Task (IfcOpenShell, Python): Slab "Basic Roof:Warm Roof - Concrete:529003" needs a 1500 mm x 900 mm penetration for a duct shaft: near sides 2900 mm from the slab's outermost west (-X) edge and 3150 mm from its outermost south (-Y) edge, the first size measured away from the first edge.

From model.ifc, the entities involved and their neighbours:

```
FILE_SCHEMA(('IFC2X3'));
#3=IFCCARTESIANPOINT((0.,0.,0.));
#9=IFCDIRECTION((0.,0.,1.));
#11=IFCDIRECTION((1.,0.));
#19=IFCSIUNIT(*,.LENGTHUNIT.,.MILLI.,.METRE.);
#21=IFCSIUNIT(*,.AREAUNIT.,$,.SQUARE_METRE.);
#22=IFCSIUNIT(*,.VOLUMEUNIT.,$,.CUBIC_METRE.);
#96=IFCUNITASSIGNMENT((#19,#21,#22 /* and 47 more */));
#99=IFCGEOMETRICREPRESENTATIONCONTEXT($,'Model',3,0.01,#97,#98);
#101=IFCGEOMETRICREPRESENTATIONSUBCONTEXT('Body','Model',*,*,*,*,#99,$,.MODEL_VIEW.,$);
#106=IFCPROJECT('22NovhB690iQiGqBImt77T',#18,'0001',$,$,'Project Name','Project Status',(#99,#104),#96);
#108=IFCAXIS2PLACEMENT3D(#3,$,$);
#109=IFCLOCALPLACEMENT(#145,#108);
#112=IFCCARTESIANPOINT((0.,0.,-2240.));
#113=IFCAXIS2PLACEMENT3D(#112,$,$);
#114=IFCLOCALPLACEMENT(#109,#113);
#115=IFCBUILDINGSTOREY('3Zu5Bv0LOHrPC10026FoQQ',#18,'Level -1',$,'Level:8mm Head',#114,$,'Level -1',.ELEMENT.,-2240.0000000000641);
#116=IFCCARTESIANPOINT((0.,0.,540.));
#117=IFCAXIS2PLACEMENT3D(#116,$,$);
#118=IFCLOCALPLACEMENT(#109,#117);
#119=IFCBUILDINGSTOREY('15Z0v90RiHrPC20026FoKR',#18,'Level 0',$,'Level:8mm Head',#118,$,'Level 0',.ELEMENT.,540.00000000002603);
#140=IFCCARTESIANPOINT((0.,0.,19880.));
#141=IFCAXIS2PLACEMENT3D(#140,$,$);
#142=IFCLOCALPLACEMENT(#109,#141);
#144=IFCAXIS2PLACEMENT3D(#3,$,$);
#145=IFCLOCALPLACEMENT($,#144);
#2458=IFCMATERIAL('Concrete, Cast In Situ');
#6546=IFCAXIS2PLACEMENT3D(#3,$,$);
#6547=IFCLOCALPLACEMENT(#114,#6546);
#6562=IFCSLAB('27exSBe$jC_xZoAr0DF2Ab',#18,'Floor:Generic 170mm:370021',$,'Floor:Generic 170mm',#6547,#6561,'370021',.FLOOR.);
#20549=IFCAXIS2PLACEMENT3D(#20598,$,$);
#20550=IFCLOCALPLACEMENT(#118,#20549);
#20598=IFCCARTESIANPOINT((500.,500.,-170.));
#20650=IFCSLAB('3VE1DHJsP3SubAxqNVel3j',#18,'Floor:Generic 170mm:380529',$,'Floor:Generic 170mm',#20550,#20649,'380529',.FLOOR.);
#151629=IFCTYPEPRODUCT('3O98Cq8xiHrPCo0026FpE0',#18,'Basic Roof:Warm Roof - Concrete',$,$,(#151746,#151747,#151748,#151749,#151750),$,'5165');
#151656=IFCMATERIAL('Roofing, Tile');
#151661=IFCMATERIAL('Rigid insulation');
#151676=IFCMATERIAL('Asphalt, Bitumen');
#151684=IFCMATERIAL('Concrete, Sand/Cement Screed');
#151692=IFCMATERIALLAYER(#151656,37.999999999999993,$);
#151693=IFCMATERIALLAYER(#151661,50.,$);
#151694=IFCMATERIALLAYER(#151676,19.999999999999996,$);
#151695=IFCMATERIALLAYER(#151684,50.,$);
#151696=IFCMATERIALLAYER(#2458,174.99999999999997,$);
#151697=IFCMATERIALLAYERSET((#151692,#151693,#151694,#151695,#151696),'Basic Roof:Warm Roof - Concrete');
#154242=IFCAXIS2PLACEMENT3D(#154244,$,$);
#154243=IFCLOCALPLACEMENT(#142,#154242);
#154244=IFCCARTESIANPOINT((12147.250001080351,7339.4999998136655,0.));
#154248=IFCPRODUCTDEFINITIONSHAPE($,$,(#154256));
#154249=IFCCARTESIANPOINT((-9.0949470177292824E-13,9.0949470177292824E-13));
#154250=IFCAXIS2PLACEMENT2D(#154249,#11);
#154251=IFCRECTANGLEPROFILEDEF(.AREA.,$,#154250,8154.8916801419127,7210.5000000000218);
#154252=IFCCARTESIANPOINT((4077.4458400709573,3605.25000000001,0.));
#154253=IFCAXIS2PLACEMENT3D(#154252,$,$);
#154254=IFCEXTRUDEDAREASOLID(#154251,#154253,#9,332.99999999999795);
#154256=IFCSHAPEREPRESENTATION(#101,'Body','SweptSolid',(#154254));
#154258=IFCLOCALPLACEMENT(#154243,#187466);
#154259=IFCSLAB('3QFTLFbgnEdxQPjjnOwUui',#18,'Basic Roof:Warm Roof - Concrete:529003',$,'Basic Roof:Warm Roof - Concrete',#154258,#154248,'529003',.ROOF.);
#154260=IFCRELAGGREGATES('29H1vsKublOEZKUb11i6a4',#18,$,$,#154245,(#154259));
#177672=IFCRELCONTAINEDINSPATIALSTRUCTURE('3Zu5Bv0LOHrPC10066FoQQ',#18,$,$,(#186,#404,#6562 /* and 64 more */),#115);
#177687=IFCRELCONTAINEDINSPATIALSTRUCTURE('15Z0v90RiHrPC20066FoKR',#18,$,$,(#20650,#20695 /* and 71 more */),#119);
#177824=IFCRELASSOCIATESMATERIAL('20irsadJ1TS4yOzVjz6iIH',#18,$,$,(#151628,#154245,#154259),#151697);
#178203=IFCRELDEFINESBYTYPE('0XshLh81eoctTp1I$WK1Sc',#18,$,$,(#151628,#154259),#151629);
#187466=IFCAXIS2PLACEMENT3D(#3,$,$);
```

```python
import numpy as np
import ifcopenshell
import ifcopenshell.api.feature
import ifcopenshell.api.geometry
import ifcopenshell.api.root
import ifcopenshell.geom
import ifcopenshell.util.placement
import ifcopenshell.util.representation
import ifcopenshell.util.shape
import ifcopenshell.util.unit

model = ifcopenshell.open("model.ifc")
unit_scale = ifcopenshell.util.unit.calculate_unit_scale(model)
settings = ifcopenshell.geom.settings()


def volume(element):
    """Net volume in cubic metres, openings subtracted."""
    shape = ifcopenshell.geom.create_shape(settings, element)
    return ifcopenshell.util.shape.get_volume(shape.geometry)


slab = model.by_id(154259)
before = volume(slab)

# Extent in the slab's own axes, in metres. The edges named are its -X and -Y sides.
slab_shape = ifcopenshell.geom.create_shape(settings, slab)
vertices = ifcopenshell.util.shape.get_vertices(slab_shape.geometry)
x_min, y_min, bottom = vertices.min(axis=0)
top = vertices[:, 2].max()

opening = ifcopenshell.api.root.create_entity(model, ifc_class="IfcOpeningElement", name="Duct shaft opening")
context = ifcopenshell.util.representation.get_context(model, "Model", "Body", "MODEL_VIEW")
width, depth = 1.5, 0.9
outline = [(0.0, 0.0), (width, 0.0), (width, depth), (0.0, depth), (0.0, 0.0)]
# Overshoot both faces by 50 mm so the cut is clean.
shape = ifcopenshell.api.geometry.add_slab_representation(
    model, context=context, depth=top - bottom + 0.1, polyline=outline
)
ifcopenshell.api.geometry.assign_representation(model, product=opening, representation=shape)

matrix = ifcopenshell.util.placement.get_local_placement(slab.ObjectPlacement)
matrix[:, 3] = matrix @ np.append(np.array([x_min + 2.9, y_min + 3.15, bottom - 0.05]) / unit_scale, 1.0)
ifcopenshell.api.geometry.edit_object_placement(model, product=opening, matrix=matrix, is_si=False)
ifcopenshell.api.feature.add_feature(model, feature=opening, element=slab)

after = volume(slab)

print(f"slab volume {before:.3f} -> {after:.3f} m3")

model.write("model_updated.ifc")
```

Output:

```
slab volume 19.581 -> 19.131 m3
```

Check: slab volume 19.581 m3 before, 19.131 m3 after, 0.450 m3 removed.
